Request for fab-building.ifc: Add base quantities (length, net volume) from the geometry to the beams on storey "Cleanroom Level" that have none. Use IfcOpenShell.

First a look at what the model holds.

```python
import ifcopenshell
import ifcopenshell.util.element
import ifcopenshell.util.unit

model = ifcopenshell.open("fab-building.ifc")
print(model.schema)
for unit_type in ("LENGTHUNIT", "AREAUNIT", "VOLUMEUNIT"):
    print(unit_type, ifcopenshell.util.unit.calculate_unit_scale(model, unit_type))
storey = next(s for s in model.by_type("IfcBuildingStorey") if s.Name == "Cleanroom Level")
beams = [e for e in ifcopenshell.util.element.get_decomposition(storey) if e.is_a("IfcBeam")]
for e in sorted(beams, key=lambda e: e.id()):
    print(e.id(), e.is_a(), e.Name, list(ifcopenshell.util.element.get_psets(e, qtos_only=True)), sep=" | ")
```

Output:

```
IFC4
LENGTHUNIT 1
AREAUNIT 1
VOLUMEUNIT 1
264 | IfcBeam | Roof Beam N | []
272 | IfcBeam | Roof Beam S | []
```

```python
import ifcopenshell
import ifcopenshell.api.pset
import ifcopenshell.geom
import ifcopenshell.util.element
import ifcopenshell.util.shape
import ifcopenshell.util.unit

model = ifcopenshell.open("fab-building.ifc")
unit_scale = ifcopenshell.util.unit.calculate_unit_scale(model)
volume_scale = ifcopenshell.util.unit.calculate_unit_scale(model, "VOLUMEUNIT")
settings = ifcopenshell.geom.settings()

storey = next(s for s in model.by_type("IfcBuildingStorey") if s.Name == "Cleanroom Level")
beams = [e for e in ifcopenshell.util.element.get_decomposition(storey) if e.is_a("IfcBeam")]

for e in sorted(beams, key=lambda e: e.id()):
    if ifcopenshell.util.element.get_psets(e, qtos_only=True, should_inherit=False):
        continue
    # Geometry comes back in metres, in the element's own axes.
    shape = ifcopenshell.geom.create_shape(settings, e)
    values = {
        "Length": ifcopenshell.util.shape.get_max_xyz(shape.geometry) / unit_scale,
        "NetVolume": ifcopenshell.util.shape.get_volume(shape.geometry) / volume_scale,
    }
    qto = ifcopenshell.api.pset.add_qto(model, product=e, name="Qto_BeamBaseQuantities")
    ifcopenshell.api.pset.edit_qto(model, qto=qto, properties=values)
    print(e.id(), {k: round(v, 3) for k, v in values.items()})

model.write("fab-building_v2.ifc")
```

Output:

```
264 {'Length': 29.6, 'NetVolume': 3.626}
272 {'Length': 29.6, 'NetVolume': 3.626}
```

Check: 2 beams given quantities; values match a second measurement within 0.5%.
